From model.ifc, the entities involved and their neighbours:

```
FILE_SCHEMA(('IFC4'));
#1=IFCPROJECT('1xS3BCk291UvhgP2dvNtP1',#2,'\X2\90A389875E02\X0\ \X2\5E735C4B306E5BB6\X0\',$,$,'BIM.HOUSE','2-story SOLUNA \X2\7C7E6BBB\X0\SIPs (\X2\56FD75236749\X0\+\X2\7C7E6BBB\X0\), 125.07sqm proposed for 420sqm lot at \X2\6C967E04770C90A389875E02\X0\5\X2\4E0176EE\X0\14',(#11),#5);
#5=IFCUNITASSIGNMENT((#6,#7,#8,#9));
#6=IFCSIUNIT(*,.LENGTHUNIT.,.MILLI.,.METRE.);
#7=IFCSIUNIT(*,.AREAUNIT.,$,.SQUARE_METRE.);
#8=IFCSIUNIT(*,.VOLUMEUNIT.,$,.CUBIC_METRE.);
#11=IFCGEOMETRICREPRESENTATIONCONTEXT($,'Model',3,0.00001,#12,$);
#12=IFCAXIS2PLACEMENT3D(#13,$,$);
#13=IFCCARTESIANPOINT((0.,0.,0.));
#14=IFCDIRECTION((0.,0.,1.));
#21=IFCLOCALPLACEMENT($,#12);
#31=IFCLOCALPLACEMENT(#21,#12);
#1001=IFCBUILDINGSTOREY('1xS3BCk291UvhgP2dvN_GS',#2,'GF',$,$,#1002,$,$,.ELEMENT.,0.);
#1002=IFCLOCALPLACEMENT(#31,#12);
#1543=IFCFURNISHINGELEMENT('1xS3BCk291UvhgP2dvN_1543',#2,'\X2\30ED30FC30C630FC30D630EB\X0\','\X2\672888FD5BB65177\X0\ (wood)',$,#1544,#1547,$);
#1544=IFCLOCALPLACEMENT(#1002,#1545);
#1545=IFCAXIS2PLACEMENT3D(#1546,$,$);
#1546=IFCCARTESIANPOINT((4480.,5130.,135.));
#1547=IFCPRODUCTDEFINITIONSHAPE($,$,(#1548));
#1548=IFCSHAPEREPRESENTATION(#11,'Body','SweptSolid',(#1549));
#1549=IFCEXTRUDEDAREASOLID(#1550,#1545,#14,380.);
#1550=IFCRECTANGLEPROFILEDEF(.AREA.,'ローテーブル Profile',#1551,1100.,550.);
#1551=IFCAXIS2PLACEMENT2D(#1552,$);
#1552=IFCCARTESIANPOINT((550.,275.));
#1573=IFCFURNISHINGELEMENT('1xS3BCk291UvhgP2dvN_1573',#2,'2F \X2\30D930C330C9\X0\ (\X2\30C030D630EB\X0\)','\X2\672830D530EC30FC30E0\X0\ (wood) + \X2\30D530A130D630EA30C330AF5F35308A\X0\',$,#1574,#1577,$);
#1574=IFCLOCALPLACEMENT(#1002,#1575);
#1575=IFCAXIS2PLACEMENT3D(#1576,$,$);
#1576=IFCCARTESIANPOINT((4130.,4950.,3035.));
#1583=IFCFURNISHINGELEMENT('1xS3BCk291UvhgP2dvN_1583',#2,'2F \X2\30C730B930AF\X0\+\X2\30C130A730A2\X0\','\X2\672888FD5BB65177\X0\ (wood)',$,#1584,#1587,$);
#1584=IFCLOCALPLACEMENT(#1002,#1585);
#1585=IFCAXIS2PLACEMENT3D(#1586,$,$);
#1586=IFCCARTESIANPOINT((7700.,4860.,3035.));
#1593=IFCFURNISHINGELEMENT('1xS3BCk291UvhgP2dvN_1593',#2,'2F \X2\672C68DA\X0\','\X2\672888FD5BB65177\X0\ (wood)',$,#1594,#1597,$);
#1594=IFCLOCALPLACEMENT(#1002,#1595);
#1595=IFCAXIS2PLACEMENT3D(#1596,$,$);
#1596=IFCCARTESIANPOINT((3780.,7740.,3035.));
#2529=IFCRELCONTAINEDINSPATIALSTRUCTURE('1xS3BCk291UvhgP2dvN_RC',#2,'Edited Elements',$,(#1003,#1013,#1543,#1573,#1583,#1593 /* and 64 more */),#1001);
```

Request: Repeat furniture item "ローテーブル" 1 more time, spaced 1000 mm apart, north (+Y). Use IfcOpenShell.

```python
import numpy as np
import ifcopenshell
import ifcopenshell.api.geometry
import ifcopenshell.api.root
import ifcopenshell.util.element
import ifcopenshell.util.placement

model = ifcopenshell.open("model.ifc")


def reuse_history(source, copy):
    """copy_class also copies each property set's owner history, people and application; keep the originals."""
    for rel in copy.IsDefinedBy:
        if rel.is_a("IfcRelDefinesByProperties") and (history := rel.RelatingPropertyDefinition.OwnerHistory):
            rel.RelatingPropertyDefinition.OwnerHistory = source.OwnerHistory
            ifcopenshell.util.element.remove_deep2(model, history)


source = model.by_guid("1xS3BCk291UvhgP2dvN_1543")
base = ifcopenshell.util.placement.get_local_placement(source.ObjectPlacement)
step = np.array([0.0, 1.0, 0.0]) * 1000.0

for i in range(1, 2):
    copy = ifcopenshell.api.root.copy_class(model, product=source)
    copy.Representation = ifcopenshell.util.element.copy_deep(
        model, source.Representation, exclude=["IfcGeometricRepresentationContext", "IfcRepresentationMap"]
    )
    reuse_history(source, copy)
    matrix = base.copy()
    matrix[:3, 3] += i * step
    print("added at", matrix[:3, 3].round(3) + 0.0)
    ifcopenshell.api.geometry.edit_object_placement(model, product=copy, matrix=matrix, is_si=False)

model.write("model_updated.ifc")
```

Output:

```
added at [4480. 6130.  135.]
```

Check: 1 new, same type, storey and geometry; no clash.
